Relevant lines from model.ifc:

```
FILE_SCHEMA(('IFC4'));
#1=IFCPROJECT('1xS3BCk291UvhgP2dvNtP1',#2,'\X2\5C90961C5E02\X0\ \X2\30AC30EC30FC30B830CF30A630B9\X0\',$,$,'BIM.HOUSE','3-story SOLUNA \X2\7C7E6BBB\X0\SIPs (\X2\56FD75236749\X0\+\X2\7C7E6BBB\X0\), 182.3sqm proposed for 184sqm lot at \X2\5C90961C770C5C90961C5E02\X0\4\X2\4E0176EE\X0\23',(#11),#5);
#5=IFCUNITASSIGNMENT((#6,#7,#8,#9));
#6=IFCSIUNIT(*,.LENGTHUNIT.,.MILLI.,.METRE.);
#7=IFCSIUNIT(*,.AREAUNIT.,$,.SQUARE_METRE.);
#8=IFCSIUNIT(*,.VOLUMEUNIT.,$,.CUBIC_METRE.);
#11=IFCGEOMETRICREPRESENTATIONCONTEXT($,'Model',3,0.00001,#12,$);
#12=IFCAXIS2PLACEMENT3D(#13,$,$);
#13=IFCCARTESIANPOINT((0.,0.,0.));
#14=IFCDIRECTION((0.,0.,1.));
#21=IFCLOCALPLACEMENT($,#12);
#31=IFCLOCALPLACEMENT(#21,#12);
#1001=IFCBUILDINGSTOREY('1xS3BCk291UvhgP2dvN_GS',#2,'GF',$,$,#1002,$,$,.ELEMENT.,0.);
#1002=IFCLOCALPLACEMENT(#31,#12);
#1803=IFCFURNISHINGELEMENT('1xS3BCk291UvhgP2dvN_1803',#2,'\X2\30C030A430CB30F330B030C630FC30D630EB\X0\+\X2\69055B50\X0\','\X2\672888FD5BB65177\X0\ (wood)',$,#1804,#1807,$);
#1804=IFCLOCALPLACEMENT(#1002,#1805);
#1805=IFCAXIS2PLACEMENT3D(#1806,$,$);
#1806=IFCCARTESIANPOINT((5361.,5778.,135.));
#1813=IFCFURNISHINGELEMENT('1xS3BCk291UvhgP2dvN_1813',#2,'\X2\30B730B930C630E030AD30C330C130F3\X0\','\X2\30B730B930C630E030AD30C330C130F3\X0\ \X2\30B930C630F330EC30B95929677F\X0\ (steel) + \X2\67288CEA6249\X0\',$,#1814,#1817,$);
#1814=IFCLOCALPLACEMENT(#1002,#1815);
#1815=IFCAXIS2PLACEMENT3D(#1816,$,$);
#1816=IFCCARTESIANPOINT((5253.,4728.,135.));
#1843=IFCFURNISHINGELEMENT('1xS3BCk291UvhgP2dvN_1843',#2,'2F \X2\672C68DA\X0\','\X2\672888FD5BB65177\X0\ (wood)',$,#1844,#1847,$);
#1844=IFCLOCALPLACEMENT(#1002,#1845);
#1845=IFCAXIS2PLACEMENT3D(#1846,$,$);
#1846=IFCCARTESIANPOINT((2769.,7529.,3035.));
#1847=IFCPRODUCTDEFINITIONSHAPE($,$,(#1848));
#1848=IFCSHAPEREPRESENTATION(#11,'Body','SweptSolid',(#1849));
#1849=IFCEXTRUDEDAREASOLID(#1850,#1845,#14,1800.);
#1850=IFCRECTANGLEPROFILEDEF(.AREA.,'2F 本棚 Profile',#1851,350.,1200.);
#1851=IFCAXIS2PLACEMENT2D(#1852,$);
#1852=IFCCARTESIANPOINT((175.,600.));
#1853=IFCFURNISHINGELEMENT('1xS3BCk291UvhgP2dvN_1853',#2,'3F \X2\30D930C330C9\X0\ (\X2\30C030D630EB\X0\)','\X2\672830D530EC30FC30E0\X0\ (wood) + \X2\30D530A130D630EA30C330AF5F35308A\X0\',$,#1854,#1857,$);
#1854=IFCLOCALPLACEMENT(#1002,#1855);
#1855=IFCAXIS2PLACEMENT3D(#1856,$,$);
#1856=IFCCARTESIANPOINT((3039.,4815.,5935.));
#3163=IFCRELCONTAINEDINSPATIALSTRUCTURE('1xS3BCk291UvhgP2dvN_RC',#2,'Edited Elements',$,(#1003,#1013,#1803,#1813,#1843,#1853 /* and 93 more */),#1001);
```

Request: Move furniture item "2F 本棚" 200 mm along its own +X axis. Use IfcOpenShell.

```python
import ifcopenshell
import ifcopenshell.api.geometry
import ifcopenshell.util.placement
import ifcopenshell.util.unit

model = ifcopenshell.open("model.ifc")
unit_scale = ifcopenshell.util.unit.calculate_unit_scale(model)

item = model.by_guid("1xS3BCk291UvhgP2dvN_1843")
matrix = ifcopenshell.util.placement.get_local_placement(item.ObjectPlacement)
matrix[:3, 3] += matrix[:3, 0] * 0.2 / unit_scale
ifcopenshell.api.geometry.edit_object_placement(model, product=item, matrix=matrix, is_si=False)

print(ifcopenshell.util.placement.get_local_placement(item.ObjectPlacement).round(3) + 0.0)

model.write("model_edited.ifc")
```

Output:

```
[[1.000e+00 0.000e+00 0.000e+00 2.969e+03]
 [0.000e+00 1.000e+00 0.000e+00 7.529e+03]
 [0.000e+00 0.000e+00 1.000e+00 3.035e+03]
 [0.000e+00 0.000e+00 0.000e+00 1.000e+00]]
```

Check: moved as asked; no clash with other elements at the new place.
